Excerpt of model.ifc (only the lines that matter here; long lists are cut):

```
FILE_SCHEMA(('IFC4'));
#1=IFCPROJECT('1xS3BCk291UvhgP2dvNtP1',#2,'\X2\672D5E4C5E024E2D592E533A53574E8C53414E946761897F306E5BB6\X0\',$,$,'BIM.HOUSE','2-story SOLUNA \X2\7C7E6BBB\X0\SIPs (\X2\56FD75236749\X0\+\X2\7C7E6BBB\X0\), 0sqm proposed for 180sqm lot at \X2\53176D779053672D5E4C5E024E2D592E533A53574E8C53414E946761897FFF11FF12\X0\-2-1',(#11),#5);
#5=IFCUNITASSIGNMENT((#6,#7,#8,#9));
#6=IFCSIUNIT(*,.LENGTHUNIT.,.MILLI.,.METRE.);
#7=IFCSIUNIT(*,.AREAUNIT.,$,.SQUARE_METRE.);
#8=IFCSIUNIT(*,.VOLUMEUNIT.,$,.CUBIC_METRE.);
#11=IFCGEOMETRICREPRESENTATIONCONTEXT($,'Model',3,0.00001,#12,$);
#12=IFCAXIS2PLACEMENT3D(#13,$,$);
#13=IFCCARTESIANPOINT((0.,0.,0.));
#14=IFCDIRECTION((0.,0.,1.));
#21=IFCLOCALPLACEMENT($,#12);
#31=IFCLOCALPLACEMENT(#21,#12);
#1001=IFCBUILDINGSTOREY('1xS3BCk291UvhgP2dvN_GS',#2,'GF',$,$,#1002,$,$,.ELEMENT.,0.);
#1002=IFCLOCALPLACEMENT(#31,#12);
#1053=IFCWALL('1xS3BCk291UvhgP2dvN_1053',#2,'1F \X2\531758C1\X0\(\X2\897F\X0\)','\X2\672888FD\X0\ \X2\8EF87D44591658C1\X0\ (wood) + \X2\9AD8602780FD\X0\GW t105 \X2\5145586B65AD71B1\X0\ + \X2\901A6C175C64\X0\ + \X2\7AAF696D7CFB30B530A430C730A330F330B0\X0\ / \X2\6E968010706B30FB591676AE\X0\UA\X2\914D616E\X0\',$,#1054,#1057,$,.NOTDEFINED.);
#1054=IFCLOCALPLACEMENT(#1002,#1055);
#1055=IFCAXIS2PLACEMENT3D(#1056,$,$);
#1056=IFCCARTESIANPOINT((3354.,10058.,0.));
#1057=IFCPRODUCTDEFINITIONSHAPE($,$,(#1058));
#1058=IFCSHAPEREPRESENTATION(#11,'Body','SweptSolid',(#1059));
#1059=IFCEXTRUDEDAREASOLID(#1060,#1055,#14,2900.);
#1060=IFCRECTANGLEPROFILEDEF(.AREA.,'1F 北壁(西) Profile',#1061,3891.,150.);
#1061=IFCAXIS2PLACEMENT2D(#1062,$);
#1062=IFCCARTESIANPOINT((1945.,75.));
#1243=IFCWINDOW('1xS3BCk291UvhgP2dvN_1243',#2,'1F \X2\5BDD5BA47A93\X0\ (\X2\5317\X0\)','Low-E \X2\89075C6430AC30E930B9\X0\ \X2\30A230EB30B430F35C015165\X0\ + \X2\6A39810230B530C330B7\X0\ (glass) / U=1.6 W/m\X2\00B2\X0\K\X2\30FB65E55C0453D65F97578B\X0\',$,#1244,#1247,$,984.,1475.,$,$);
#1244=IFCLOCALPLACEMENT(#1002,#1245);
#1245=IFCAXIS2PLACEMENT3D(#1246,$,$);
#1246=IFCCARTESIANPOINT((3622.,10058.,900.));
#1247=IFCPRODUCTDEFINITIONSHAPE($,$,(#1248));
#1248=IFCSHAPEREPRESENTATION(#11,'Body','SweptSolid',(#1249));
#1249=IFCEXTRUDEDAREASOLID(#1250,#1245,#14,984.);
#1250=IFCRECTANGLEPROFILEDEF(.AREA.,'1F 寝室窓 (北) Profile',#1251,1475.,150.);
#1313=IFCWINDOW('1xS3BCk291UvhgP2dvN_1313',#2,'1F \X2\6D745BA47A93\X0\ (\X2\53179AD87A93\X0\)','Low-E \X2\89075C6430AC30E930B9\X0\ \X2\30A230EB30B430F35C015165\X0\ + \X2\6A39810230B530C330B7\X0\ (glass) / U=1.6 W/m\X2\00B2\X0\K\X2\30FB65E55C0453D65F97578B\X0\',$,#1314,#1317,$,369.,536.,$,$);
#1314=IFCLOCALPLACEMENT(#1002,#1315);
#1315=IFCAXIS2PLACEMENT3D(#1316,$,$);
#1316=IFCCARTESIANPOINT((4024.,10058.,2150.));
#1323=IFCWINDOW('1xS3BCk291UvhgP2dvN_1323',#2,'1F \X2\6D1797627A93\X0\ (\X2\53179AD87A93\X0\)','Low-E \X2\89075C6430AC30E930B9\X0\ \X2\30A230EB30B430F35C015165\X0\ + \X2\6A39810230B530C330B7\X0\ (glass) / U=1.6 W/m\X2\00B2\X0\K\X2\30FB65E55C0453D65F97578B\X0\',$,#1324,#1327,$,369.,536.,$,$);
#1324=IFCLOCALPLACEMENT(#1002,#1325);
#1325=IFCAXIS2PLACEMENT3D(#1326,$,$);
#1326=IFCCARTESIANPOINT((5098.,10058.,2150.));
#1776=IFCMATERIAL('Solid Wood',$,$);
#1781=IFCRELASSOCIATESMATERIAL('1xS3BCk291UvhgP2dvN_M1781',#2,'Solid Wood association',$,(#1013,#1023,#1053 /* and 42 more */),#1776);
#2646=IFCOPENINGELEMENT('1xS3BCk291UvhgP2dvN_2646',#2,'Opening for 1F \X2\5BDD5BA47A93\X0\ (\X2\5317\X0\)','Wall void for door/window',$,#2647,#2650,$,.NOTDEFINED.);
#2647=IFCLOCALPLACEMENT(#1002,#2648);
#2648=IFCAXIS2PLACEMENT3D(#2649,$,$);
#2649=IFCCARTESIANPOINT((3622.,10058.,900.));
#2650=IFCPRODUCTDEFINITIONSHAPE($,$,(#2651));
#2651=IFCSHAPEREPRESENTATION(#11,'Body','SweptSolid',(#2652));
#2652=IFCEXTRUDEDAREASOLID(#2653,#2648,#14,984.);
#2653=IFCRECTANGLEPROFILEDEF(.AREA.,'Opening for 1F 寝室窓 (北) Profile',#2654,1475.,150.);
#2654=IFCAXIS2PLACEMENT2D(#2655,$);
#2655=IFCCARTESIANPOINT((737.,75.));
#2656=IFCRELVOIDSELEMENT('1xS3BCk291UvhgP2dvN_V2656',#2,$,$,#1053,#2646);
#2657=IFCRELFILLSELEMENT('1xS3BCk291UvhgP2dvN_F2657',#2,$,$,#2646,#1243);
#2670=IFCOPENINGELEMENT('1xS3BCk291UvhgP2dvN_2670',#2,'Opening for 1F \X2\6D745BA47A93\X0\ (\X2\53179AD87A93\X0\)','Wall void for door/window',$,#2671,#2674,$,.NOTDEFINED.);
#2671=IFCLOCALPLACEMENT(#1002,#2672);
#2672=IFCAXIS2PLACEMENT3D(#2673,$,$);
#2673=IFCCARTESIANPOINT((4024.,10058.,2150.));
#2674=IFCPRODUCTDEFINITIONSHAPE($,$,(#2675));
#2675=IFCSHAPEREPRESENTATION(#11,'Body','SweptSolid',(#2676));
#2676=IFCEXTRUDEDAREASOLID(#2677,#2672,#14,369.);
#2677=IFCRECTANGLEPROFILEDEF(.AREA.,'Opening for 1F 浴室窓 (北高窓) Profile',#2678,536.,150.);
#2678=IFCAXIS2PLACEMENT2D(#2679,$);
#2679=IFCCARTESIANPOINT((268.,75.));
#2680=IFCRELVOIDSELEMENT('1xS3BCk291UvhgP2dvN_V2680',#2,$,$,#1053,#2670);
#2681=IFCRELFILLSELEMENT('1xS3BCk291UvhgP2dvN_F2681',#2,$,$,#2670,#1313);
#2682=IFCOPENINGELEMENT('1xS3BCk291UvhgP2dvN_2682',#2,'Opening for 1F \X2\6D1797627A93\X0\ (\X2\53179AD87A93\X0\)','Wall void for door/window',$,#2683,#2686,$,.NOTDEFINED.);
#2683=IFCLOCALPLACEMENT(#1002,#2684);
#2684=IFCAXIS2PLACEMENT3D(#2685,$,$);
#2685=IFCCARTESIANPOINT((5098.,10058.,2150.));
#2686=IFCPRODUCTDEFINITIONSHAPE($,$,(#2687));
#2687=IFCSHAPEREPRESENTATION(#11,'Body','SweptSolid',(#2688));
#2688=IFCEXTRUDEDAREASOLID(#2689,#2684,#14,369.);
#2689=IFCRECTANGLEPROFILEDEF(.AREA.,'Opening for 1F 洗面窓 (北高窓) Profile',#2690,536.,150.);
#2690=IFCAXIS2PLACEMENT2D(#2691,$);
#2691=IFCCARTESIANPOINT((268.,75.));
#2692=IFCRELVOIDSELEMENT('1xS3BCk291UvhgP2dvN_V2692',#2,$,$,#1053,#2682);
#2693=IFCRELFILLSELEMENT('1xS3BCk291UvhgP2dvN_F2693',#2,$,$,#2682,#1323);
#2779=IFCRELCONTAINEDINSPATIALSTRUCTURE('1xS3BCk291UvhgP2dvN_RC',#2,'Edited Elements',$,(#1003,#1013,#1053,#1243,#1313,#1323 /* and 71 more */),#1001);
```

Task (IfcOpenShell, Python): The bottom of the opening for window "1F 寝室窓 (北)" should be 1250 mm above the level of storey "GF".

```python
import numpy as np
import ifcopenshell
import ifcopenshell.api.geometry
import ifcopenshell.geom
import ifcopenshell.util.element
import ifcopenshell.util.placement
import ifcopenshell.util.shape
import ifcopenshell.util.unit

model = ifcopenshell.open("model.ifc")
unit_scale = ifcopenshell.util.unit.calculate_unit_scale(model)

window = model.by_guid("1xS3BCk291UvhgP2dvN_1243")
opening = window.FillsVoids[0].RelatingOpeningElement
storey = ifcopenshell.util.element.get_container(window, ifc_class="IfcBuildingStorey")
level = ifcopenshell.util.placement.get_local_placement(storey.ObjectPlacement)[2, 3]

# The opening's origin need not be at the sill, so measure its lowest point.
shape = ifcopenshell.geom.create_shape(ifcopenshell.geom.settings(), opening)
bottom = ifcopenshell.util.shape.get_shape_bottom_elevation(shape, shape.geometry) / unit_scale
dz = level + 1250.0 - bottom

shift = np.array([0.0, 0.0, dz])
# The window is not placed relative to its opening, so move both.
for product in (opening, window):
    matrix = ifcopenshell.util.placement.get_local_placement(product.ObjectPlacement)
    matrix[:3, 3] += shift
    ifcopenshell.api.geometry.edit_object_placement(model, product=product, matrix=matrix, is_si=False)

print(f"moved by {dz * unit_scale:+.3f} m")

model.write("model_rev.ifc")
```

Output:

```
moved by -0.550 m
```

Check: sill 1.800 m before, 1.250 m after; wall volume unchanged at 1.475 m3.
